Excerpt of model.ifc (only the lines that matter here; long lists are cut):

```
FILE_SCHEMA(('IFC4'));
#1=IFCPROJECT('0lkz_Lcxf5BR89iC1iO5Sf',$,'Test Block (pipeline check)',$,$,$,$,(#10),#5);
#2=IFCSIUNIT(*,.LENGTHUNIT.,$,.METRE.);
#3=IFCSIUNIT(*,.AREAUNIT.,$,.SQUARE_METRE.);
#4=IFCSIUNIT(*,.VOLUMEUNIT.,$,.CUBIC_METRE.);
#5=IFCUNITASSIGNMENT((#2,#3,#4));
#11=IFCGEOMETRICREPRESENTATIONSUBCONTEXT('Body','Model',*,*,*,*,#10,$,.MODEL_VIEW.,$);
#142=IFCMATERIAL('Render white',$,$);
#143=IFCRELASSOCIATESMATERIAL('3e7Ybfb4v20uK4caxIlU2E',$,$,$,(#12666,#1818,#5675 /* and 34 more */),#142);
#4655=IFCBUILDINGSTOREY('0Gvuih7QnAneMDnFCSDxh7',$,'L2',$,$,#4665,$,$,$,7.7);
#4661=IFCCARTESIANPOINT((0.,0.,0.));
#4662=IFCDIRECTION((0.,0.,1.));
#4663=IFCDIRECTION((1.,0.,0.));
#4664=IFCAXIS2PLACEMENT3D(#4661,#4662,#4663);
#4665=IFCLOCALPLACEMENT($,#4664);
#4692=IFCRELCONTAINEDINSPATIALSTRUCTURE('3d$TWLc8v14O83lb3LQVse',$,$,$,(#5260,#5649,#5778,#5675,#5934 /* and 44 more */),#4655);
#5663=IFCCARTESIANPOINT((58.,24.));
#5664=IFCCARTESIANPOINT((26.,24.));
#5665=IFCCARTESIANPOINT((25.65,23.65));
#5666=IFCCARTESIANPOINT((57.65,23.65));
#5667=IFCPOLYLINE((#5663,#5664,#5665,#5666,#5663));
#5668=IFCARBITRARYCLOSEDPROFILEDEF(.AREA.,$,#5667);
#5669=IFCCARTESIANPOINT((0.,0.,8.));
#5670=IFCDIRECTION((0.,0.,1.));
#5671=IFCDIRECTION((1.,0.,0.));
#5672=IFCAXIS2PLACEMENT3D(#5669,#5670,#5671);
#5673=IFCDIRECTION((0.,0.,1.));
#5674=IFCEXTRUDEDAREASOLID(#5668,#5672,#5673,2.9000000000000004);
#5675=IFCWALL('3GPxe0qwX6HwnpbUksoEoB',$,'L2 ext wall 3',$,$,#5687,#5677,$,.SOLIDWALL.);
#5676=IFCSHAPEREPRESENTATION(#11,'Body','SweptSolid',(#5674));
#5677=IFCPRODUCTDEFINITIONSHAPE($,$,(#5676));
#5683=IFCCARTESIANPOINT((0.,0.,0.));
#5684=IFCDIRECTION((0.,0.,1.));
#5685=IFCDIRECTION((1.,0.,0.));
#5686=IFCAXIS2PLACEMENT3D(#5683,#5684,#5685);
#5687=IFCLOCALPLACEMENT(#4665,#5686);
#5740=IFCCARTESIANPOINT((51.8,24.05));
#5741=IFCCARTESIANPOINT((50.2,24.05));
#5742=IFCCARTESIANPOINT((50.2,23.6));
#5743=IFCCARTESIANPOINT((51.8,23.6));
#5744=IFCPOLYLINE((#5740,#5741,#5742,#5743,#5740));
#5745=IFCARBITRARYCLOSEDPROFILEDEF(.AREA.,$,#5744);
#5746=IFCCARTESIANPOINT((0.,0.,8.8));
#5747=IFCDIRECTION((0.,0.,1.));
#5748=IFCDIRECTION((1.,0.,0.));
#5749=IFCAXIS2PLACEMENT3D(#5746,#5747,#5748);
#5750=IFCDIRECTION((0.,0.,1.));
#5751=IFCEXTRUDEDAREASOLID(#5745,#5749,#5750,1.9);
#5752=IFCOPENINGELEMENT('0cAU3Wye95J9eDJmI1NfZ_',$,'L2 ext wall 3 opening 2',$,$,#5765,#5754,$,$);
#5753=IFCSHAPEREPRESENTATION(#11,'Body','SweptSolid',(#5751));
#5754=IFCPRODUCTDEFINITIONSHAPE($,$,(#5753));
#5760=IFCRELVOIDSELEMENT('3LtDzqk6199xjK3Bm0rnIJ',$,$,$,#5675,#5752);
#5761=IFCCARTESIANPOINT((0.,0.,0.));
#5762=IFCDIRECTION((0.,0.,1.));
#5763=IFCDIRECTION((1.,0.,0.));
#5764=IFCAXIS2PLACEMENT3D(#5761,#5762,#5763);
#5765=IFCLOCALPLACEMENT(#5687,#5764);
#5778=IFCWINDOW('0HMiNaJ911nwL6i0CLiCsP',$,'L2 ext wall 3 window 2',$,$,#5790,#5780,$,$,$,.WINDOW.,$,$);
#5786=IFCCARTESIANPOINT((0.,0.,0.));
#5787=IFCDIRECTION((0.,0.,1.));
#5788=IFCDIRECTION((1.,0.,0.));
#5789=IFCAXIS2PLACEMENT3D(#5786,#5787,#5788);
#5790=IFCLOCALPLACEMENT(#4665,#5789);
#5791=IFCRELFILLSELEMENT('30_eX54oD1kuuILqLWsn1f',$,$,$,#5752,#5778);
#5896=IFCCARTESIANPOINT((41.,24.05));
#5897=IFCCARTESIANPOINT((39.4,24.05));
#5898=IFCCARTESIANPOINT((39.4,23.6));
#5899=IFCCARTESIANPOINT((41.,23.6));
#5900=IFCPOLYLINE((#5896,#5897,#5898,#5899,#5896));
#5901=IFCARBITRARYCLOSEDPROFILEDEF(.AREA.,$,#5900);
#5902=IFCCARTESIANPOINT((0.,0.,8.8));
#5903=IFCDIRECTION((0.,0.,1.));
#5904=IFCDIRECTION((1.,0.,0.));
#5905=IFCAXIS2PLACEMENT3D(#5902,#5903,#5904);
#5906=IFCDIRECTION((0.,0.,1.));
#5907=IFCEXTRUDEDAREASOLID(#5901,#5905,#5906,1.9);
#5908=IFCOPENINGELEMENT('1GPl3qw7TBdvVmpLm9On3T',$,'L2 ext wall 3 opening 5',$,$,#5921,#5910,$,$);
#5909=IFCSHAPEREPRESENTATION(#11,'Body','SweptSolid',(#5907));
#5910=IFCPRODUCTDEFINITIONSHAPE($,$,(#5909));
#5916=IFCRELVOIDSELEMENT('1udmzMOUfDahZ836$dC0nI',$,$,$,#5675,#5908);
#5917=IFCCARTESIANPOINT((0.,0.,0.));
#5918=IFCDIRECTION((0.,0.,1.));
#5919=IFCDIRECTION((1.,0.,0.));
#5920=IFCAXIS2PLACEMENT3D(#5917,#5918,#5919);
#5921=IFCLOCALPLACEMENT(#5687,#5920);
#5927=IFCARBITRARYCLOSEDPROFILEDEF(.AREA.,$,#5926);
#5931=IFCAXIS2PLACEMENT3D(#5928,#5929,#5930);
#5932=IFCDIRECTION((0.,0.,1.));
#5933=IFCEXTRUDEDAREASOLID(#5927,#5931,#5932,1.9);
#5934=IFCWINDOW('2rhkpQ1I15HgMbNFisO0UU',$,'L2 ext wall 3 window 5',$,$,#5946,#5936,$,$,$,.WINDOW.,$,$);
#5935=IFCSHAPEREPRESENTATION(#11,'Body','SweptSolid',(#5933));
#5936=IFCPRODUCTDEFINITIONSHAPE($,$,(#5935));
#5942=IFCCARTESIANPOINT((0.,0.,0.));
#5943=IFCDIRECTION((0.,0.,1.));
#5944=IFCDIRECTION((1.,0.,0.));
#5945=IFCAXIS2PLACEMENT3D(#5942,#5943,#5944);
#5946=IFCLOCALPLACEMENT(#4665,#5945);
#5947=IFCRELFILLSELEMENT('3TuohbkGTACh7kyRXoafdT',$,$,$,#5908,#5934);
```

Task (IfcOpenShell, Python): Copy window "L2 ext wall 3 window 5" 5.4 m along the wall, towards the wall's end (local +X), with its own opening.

```python
import ifcopenshell
import ifcopenshell.api.feature
import ifcopenshell.api.geometry
import ifcopenshell.api.root
import ifcopenshell.geom
import ifcopenshell.util.element
import ifcopenshell.util.placement
import ifcopenshell.util.shape

model = ifcopenshell.open("model.ifc")
settings = ifcopenshell.geom.settings()


def volume(element):
    """Net volume in cubic metres, openings subtracted."""
    shape = ifcopenshell.geom.create_shape(settings, element)
    return ifcopenshell.util.shape.get_volume(shape.geometry)


window = model.by_guid("2rhkpQ1I15HgMbNFisO0UU")
opening = window.FillsVoids[0].RelatingOpeningElement
wall = opening.VoidsElements[0].RelatingBuildingElement
before = volume(wall)
shift = ifcopenshell.util.placement.get_local_placement(wall.ObjectPlacement)[:3, 0] * 5.4

# copy_class copies the void relationship, type, container and properties, but no geometry.
new_opening = ifcopenshell.api.root.copy_class(model, product=opening)
new_opening.Representation = ifcopenshell.util.element.copy_deep(
    model, opening.Representation, exclude=["IfcGeometricRepresentationContext", "IfcRepresentationMap"]
)
new_window = ifcopenshell.api.root.copy_class(model, product=window)
new_window.Representation = ifcopenshell.util.element.copy_deep(
    model, window.Representation, exclude=["IfcGeometricRepresentationContext", "IfcRepresentationMap"]
)
ifcopenshell.api.feature.add_filling(model, opening=new_opening, element=new_window)

for old, new in ((opening, new_opening), (window, new_window)):
    matrix = ifcopenshell.util.placement.get_local_placement(old.ObjectPlacement)
    matrix[:3, 3] += shift
    ifcopenshell.api.geometry.edit_object_placement(model, product=new, matrix=matrix, is_si=False)

after = volume(wall)

print(f"wall volume {before:.3f} -> {after:.3f} m3")

model.write("model_edited.ifc")
```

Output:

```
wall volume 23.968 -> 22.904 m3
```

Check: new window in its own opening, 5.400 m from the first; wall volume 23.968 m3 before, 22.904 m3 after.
